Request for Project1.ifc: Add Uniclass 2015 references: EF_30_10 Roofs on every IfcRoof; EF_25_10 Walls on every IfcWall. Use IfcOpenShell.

First a look at what the model holds.

```python
import ifcopenshell

model = ifcopenshell.open("Project1.ifc")
print(model.schema)
print("classifications:", [c.Name for c in model.by_type("IfcClassification")])
for ifc_class in ("IfcDoor", "IfcRoof", "IfcStair", "IfcWall", "IfcWindow"):
    print(ifc_class, len(model.by_type(ifc_class)))
```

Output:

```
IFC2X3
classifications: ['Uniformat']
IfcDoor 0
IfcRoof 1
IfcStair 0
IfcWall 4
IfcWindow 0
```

```python
import ifcopenshell
import ifcopenshell.api.classification

model = ifcopenshell.open("Project1.ifc")

# IFC2X3 requires Source and Edition and has no link from the project to the system.
system = model.create_entity("IfcClassification", Source="NBS", Edition="2015", Name="Uniclass 2015")

codes = {
    "IfcRoof": ("EF_30_10", "Roofs"),
    "IfcWall": ("EF_25_10", "Walls"),
}
for ifc_class, (code, name) in codes.items():
    products = model.by_type(ifc_class)
    ifcopenshell.api.classification.add_reference(
        model, products=products, classification=system, identification=code, name=name
    )
    print(code, len(products))

model.write("Project1_edited.ifc")
```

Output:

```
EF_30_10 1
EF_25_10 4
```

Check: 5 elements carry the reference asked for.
